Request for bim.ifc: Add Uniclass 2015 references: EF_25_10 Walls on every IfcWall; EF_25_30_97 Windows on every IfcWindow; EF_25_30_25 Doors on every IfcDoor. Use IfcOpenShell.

First a look at what the model holds.

```python
import ifcopenshell

model = ifcopenshell.open("bim.ifc")
print(model.schema)
print("classifications:", [c.Name for c in model.by_type("IfcClassification")])
for ifc_class in ("IfcDoor", "IfcRoof", "IfcStair", "IfcWall", "IfcWindow"):
    print(ifc_class, len(model.by_type(ifc_class)))
```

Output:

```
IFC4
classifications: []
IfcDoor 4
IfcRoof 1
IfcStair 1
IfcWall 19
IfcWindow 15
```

```python
import ifcopenshell
import ifcopenshell.api.classification

model = ifcopenshell.open("bim.ifc")

system = ifcopenshell.api.classification.add_classification(model, classification="Uniclass 2015")

codes = {
    "IfcWall": ("EF_25_10", "Walls"),
    "IfcWindow": ("EF_25_30_97", "Windows"),
    "IfcDoor": ("EF_25_30_25", "Doors"),
}
for ifc_class, (code, name) in codes.items():
    products = model.by_type(ifc_class)
    ifcopenshell.api.classification.add_reference(
        model, products=products, classification=system, identification=code, name=name
    )
    print(code, len(products))

model.write("bim_updated.ifc")
```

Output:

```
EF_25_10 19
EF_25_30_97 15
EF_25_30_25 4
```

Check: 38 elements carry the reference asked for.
